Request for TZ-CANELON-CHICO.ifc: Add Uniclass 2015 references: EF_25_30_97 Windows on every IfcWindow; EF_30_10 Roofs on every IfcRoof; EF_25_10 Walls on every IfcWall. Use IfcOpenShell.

First a look at what the model holds.

```python
import ifcopenshell

model = ifcopenshell.open("TZ-CANELON-CHICO.ifc")
print(model.schema)
print("classifications:", [c.Name for c in model.by_type("IfcClassification")])
for ifc_class in ("IfcDoor", "IfcRoof", "IfcStair", "IfcWall", "IfcWindow"):
    print(ifc_class, len(model.by_type(ifc_class)))
```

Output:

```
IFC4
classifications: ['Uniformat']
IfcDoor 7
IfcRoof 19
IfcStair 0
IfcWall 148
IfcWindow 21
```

```python
import ifcopenshell
import ifcopenshell.api.classification

model = ifcopenshell.open("TZ-CANELON-CHICO.ifc")

system = ifcopenshell.api.classification.add_classification(model, classification="Uniclass 2015")

codes = {
    "IfcWindow": ("EF_25_30_97", "Windows"),
    "IfcRoof": ("EF_30_10", "Roofs"),
    "IfcWall": ("EF_25_10", "Walls"),
}
for ifc_class, (code, name) in codes.items():
    products = model.by_type(ifc_class)
    ifcopenshell.api.classification.add_reference(
        model, products=products, classification=system, identification=code, name=name
    )
    print(code, len(products))

model.write("TZ-CANELON-CHICO_v2.ifc")
```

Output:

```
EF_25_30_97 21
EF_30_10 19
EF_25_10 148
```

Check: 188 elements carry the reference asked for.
